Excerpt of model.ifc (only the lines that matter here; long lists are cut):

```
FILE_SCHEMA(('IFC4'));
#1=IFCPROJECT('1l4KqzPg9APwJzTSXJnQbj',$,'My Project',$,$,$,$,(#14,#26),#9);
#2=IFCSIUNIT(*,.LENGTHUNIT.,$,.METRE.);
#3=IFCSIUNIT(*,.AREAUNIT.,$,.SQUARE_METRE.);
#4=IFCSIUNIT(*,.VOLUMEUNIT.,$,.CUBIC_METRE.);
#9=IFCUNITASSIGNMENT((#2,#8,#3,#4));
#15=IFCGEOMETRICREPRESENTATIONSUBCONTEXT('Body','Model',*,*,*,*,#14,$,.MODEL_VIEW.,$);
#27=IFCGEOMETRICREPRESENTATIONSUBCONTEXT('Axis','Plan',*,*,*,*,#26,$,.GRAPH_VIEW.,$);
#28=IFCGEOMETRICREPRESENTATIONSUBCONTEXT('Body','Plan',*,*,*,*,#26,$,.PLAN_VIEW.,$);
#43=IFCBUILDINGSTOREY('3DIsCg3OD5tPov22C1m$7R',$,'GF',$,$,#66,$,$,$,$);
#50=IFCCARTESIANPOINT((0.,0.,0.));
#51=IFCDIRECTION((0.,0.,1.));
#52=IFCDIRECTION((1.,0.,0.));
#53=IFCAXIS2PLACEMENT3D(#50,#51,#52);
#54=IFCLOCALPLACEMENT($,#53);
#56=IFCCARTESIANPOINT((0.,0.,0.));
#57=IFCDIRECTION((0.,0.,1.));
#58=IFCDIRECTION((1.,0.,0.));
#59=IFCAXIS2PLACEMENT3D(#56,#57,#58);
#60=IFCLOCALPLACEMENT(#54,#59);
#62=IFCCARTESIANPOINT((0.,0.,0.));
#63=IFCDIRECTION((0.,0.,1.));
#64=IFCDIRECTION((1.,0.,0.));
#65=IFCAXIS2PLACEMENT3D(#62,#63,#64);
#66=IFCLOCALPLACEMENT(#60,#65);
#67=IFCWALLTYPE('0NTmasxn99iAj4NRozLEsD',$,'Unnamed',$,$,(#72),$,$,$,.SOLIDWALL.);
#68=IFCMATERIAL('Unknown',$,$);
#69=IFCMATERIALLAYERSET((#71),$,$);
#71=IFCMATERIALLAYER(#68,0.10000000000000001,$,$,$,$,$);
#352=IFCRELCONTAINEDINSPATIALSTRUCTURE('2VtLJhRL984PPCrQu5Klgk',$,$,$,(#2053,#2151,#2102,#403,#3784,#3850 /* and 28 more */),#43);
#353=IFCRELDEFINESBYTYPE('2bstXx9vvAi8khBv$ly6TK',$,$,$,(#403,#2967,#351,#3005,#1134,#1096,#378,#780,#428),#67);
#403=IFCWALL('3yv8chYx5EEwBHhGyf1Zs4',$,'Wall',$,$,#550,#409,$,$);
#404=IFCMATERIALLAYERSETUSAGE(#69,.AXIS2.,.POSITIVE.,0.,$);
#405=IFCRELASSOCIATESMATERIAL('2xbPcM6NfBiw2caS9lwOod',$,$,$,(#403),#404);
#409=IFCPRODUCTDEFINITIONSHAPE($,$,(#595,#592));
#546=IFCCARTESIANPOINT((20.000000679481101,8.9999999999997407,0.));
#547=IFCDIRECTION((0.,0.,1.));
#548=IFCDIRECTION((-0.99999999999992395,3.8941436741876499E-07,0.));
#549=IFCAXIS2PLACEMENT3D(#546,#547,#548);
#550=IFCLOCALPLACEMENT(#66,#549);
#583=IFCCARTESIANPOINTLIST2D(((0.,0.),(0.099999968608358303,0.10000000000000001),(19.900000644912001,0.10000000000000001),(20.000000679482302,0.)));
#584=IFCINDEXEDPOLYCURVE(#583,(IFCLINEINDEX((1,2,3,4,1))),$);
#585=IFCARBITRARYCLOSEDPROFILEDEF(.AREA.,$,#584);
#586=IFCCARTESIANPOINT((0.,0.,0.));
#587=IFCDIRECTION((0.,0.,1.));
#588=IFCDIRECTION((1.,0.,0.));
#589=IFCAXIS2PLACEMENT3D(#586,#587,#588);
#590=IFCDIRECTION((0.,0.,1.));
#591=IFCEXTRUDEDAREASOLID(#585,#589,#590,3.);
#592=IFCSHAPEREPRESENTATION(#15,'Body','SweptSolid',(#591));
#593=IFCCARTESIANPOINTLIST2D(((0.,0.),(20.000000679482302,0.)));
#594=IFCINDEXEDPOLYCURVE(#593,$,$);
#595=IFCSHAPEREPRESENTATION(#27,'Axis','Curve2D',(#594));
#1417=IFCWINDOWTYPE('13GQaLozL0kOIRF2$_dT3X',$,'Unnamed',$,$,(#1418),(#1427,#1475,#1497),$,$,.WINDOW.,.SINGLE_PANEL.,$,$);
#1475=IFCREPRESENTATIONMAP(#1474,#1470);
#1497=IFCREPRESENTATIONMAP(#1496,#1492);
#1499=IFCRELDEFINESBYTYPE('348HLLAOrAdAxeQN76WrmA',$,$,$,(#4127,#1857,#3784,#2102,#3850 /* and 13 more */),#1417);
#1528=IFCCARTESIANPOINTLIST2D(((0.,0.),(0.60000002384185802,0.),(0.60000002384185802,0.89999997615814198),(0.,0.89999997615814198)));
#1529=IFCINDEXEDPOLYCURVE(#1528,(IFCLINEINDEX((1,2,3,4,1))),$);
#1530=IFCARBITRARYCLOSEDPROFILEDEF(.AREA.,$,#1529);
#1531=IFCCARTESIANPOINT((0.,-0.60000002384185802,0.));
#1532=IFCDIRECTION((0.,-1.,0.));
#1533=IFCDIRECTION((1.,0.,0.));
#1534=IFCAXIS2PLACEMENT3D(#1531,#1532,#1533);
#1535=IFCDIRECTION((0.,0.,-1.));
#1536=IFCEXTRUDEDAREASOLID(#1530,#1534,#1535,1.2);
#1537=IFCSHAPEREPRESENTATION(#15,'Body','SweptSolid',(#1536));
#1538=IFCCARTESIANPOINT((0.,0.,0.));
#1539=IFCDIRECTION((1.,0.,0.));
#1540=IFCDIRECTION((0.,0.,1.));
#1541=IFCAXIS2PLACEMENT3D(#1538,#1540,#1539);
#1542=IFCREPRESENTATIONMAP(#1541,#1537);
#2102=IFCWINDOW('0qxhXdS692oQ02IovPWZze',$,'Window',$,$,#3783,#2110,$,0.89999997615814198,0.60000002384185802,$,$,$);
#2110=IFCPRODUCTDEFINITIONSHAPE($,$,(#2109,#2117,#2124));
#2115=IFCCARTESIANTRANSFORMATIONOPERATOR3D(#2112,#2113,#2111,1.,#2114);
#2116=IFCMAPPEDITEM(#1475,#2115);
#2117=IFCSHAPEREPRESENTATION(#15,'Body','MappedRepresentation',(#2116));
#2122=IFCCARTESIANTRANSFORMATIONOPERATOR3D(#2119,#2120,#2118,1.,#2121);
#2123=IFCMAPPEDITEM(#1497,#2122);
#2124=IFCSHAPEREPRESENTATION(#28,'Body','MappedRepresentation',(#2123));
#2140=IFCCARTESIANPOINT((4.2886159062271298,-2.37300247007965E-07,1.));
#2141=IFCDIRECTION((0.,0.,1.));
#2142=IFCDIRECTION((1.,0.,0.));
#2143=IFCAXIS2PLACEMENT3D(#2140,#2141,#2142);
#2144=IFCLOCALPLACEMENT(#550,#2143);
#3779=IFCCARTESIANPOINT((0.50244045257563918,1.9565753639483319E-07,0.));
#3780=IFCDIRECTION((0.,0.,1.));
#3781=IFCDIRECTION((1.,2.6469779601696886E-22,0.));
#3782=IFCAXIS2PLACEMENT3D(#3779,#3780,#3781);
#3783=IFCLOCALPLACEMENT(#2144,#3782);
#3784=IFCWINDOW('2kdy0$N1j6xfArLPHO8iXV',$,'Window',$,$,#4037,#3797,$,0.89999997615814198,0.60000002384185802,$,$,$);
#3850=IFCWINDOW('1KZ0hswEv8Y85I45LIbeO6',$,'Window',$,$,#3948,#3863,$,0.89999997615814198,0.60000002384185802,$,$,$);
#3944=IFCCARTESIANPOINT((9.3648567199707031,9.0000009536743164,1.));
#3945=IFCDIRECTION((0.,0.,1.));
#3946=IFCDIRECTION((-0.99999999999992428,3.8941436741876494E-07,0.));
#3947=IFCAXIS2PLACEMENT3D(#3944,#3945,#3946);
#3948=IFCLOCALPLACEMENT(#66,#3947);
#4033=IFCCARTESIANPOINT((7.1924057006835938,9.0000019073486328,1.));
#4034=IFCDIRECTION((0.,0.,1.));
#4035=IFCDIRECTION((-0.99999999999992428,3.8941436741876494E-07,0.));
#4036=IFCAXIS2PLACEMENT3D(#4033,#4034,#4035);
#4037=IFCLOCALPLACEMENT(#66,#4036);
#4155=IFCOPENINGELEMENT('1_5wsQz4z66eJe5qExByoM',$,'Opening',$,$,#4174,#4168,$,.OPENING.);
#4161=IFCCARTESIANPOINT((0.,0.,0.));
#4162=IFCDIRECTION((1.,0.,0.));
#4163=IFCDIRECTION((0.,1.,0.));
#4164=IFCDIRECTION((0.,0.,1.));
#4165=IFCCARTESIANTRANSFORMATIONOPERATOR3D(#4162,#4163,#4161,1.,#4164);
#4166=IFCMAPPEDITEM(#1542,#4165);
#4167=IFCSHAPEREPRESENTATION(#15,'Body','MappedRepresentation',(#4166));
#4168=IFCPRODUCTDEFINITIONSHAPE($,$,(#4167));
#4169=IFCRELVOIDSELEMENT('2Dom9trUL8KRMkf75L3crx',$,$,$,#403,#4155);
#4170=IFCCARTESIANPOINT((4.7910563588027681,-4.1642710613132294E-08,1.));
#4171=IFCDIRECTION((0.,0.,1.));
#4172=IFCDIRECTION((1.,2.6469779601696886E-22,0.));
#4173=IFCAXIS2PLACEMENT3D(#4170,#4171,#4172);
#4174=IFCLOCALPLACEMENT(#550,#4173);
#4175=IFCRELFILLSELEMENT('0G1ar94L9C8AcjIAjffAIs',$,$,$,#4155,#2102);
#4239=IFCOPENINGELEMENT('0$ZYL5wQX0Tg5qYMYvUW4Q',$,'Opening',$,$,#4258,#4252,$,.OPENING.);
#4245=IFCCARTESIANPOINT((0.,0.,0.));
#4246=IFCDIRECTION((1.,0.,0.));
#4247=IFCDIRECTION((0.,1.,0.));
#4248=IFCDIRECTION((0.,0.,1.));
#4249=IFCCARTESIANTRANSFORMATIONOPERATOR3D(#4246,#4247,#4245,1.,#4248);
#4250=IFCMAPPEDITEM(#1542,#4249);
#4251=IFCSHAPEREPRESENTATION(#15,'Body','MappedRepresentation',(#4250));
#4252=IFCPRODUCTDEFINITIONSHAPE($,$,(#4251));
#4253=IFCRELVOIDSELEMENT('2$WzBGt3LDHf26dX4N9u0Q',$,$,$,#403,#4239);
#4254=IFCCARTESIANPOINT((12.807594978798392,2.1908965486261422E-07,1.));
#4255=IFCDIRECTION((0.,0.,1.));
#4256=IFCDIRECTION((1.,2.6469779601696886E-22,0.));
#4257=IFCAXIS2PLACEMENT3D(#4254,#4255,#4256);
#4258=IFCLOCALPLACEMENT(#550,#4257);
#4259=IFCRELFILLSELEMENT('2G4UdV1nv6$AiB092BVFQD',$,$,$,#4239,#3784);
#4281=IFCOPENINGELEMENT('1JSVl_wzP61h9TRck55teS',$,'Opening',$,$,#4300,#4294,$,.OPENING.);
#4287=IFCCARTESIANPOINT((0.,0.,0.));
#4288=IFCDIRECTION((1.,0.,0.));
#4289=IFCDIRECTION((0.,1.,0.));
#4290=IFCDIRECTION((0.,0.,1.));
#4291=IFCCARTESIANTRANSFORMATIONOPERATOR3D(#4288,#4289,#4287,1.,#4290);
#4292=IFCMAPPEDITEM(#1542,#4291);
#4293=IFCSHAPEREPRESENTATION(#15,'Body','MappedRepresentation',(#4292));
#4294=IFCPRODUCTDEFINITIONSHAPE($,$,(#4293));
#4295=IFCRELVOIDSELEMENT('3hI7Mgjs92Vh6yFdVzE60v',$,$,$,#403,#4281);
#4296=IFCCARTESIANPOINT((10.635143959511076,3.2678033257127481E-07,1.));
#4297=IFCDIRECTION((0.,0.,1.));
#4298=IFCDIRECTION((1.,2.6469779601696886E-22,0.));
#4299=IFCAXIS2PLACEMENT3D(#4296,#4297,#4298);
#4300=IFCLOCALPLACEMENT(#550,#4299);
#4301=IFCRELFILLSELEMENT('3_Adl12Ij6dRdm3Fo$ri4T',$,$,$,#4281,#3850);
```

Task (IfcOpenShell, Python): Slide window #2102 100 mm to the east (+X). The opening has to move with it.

```python
import ifcopenshell
import ifcopenshell.api.geometry
import ifcopenshell.util.placement
import ifcopenshell.util.unit

model = ifcopenshell.open("model.ifc")
unit_scale = ifcopenshell.util.unit.calculate_unit_scale(model)

window = model.by_guid("0qxhXdS692oQ02IovPWZze")
opening = window.FillsVoids[0].RelatingOpeningElement
wall = opening.VoidsElements[0].RelatingBuildingElement

wall_matrix = ifcopenshell.util.placement.get_local_placement(wall.ObjectPlacement)
shift = wall_matrix[:3, 0] * -0.1 / unit_scale
before = ifcopenshell.util.placement.get_local_placement(window.ObjectPlacement)[:3, 3].copy()

# The window is not placed relative to its opening, so move both.
for product in (opening, window):
    matrix = ifcopenshell.util.placement.get_local_placement(product.ObjectPlacement)
    matrix[:3, 3] += shift
    ifcopenshell.api.geometry.edit_object_placement(model, product=product, matrix=matrix, is_si=False)

after = ifcopenshell.util.placement.get_local_placement(window.ObjectPlacement)[:3, 3]
print("window moved by", (after - before).round(3) + 0.0)

model.write("model_updated.ifc")
```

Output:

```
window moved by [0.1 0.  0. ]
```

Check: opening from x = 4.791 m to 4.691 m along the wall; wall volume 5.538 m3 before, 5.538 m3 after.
